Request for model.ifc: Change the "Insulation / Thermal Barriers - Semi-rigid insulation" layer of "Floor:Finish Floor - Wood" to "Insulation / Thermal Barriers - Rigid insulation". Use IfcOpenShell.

First a look at what the model holds.

```python
import ifcopenshell
import ifcopenshell.util.element

model = ifcopenshell.open("model.ifc")
print(model.schema)
for layer_set in model.by_type("IfcMaterialLayerSet"):
    if layer_set.LayerSetName == "Floor:Finish Floor - Wood":
        for layer in layer_set.MaterialLayers:
            print(layer.id(), layer.Material and layer.Material.Name, layer.LayerThickness, sep=" | ")
        print(len(ifcopenshell.util.element.get_elements_by_material(model, layer_set)), "elements and types use it")
print(sorted(m.Name for m in model.by_type("IfcMaterial") if m.Name)[:60])
```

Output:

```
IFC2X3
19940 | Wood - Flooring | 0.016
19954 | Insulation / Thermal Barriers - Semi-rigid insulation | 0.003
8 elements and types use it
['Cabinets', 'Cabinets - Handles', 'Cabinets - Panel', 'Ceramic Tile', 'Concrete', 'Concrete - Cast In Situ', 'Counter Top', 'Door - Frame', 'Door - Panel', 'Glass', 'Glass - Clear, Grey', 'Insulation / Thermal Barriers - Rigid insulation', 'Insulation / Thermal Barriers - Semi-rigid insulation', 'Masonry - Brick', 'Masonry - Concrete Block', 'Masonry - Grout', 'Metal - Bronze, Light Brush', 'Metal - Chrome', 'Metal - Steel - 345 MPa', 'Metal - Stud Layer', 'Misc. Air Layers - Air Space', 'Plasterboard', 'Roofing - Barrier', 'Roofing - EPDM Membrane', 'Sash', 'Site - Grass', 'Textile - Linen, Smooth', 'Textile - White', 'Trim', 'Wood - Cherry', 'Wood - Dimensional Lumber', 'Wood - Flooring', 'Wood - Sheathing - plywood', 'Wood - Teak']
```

```python
import ifcopenshell
import ifcopenshell.api.material

model = ifcopenshell.open("model.ifc")

layer_set = next(s for s in model.by_type("IfcMaterialLayerSet") if s.LayerSetName == "Floor:Finish Floor - Wood")
layer = next(l for l in layer_set.MaterialLayers if l.Material and l.Material.Name == "Insulation / Thermal Barriers - Semi-rigid insulation")
material = next(m for m in model.by_type("IfcMaterial") if m.Name == "Insulation / Thermal Barriers - Rigid insulation")

# Point this one layer at the other material; renaming the old one would change it everywhere.
ifcopenshell.api.material.edit_layer(model, layer=layer, attributes={}, material=material)

print([l.Material.Name if l.Material else None for l in layer_set.MaterialLayers])

model.write("model_updated.ifc")
```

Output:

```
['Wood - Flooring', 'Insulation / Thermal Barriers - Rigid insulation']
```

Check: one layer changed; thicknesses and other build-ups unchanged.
